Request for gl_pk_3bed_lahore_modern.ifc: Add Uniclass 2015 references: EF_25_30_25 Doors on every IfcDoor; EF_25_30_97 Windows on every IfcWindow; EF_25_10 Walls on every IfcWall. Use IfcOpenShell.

First a look at what the model holds.

```python
import ifcopenshell

model = ifcopenshell.open("gl_pk_3bed_lahore_modern.ifc")
print(model.schema)
print("classifications:", [c.Name for c in model.by_type("IfcClassification")])
for ifc_class in ("IfcDoor", "IfcRoof", "IfcStair", "IfcWall", "IfcWindow"):
    print(ifc_class, len(model.by_type(ifc_class)))
```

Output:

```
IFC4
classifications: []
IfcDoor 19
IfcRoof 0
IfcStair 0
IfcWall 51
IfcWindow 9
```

```python
import ifcopenshell
import ifcopenshell.api.classification

model = ifcopenshell.open("gl_pk_3bed_lahore_modern.ifc")

system = ifcopenshell.api.classification.add_classification(model, classification="Uniclass 2015")

codes = {
    "IfcDoor": ("EF_25_30_25", "Doors"),
    "IfcWindow": ("EF_25_30_97", "Windows"),
    "IfcWall": ("EF_25_10", "Walls"),
}
for ifc_class, (code, name) in codes.items():
    products = model.by_type(ifc_class)
    ifcopenshell.api.classification.add_reference(
        model, products=products, classification=system, identification=code, name=name
    )
    print(code, len(products))

model.write("gl_pk_3bed_lahore_modern_updated.ifc")
```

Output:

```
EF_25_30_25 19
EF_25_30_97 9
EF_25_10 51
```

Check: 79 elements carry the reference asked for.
